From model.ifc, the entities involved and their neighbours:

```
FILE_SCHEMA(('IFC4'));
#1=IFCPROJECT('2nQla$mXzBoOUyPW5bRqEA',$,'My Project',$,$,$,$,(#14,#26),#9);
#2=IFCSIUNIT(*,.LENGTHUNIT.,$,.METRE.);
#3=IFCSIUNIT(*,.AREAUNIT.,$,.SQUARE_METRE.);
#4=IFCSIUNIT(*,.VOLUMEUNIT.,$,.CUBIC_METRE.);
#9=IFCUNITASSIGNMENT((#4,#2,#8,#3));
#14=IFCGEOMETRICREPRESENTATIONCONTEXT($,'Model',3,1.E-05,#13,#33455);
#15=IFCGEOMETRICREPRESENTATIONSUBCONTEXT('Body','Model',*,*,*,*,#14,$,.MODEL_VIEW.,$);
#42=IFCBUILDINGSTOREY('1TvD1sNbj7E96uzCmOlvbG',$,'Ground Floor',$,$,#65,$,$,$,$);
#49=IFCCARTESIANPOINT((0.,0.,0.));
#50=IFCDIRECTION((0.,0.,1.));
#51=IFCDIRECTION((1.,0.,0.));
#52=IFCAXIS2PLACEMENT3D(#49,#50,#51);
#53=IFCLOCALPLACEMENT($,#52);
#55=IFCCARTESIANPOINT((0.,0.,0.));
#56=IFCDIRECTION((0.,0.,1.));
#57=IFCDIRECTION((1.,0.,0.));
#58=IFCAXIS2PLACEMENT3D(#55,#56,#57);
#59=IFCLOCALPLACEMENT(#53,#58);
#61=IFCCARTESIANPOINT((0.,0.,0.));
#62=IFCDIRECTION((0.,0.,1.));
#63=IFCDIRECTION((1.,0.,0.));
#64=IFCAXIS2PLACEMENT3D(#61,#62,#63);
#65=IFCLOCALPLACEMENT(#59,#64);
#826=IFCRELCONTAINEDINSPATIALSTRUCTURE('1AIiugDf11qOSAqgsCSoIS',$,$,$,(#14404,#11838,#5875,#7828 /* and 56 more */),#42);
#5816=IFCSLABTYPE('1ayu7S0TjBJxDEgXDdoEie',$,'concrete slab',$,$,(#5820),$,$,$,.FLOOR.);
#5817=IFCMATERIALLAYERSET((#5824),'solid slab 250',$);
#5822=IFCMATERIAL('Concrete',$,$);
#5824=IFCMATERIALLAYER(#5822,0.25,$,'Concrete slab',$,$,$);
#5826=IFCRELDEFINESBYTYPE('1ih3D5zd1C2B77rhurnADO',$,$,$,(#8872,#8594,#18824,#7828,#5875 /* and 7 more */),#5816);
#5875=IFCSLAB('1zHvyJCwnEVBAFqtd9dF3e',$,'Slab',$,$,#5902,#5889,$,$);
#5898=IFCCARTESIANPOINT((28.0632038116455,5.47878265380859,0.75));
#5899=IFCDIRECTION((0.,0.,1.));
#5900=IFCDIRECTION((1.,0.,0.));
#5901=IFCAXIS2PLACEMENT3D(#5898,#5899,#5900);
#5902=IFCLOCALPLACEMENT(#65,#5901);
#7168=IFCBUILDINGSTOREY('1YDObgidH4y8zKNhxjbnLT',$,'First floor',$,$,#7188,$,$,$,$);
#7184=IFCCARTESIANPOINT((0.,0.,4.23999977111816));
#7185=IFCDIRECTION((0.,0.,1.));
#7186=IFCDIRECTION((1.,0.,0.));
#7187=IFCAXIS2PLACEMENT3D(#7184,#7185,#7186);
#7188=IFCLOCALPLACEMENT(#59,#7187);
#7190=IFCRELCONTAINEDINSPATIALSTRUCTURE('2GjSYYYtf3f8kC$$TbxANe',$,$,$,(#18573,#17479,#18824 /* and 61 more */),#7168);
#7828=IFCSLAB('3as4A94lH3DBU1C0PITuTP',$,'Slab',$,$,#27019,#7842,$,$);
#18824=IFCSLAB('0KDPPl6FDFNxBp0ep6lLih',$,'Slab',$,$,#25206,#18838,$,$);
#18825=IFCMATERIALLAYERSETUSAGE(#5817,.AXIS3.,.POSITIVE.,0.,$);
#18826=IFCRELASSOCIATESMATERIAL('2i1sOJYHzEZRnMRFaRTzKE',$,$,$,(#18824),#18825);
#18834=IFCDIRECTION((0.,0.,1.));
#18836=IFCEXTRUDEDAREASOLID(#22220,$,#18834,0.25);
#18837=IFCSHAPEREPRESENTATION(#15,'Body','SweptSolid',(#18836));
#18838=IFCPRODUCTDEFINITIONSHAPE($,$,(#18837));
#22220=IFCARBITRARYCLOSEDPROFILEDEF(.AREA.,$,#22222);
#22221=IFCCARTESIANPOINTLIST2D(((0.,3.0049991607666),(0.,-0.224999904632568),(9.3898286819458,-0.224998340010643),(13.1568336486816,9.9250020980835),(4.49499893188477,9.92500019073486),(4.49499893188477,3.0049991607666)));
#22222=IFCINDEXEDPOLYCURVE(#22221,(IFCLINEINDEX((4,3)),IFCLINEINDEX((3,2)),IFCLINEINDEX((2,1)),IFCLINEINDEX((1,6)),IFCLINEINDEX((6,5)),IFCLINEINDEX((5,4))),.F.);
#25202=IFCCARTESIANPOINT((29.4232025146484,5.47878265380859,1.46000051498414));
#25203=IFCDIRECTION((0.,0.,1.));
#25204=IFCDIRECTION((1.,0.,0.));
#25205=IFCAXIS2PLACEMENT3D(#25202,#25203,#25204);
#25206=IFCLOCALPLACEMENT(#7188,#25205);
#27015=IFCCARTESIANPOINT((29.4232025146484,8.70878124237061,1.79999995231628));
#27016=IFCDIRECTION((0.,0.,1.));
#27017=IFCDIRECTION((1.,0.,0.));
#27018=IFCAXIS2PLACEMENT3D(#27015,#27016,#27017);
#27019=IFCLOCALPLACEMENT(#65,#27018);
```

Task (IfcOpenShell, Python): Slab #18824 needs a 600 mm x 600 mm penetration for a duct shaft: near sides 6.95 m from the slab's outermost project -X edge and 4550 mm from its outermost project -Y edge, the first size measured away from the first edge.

```python
import numpy as np
import ifcopenshell
import ifcopenshell.api.feature
import ifcopenshell.api.geometry
import ifcopenshell.api.root
import ifcopenshell.geom
import ifcopenshell.util.placement
import ifcopenshell.util.representation
import ifcopenshell.util.shape
import ifcopenshell.util.unit

model = ifcopenshell.open("model.ifc")
unit_scale = ifcopenshell.util.unit.calculate_unit_scale(model)
settings = ifcopenshell.geom.settings()


def volume(element):
    """Net volume in cubic metres, openings subtracted."""
    shape = ifcopenshell.geom.create_shape(settings, element)
    return ifcopenshell.util.shape.get_volume(shape.geometry)


slab = model.by_guid("0KDPPl6FDFNxBp0ep6lLih")
before = volume(slab)

# Extent in the slab's own axes, in metres. The edges named are its -X and -Y sides.
slab_shape = ifcopenshell.geom.create_shape(settings, slab)
vertices = ifcopenshell.util.shape.get_vertices(slab_shape.geometry)
x_min, y_min, bottom = vertices.min(axis=0)
top = vertices[:, 2].max()

opening = ifcopenshell.api.root.create_entity(model, ifc_class="IfcOpeningElement", name="Duct shaft opening", predefined_type="OPENING")
context = ifcopenshell.util.representation.get_context(model, "Model", "Body", "MODEL_VIEW")
width, depth = 0.6, 0.6
outline = [(0.0, 0.0), (width, 0.0), (width, depth), (0.0, depth), (0.0, 0.0)]
# Overshoot both faces by 50 mm so the cut is clean.
shape = ifcopenshell.api.geometry.add_slab_representation(
    model, context=context, depth=top - bottom + 0.1, polyline=outline
)
ifcopenshell.api.geometry.assign_representation(model, product=opening, representation=shape)

matrix = ifcopenshell.util.placement.get_local_placement(slab.ObjectPlacement)
matrix[:, 3] = matrix @ np.append(np.array([x_min + 6.95, y_min + 4.55, bottom - 0.05]) / unit_scale, 1.0)
ifcopenshell.api.geometry.edit_object_placement(model, product=opening, matrix=matrix, is_si=False)
ifcopenshell.api.feature.add_feature(model, feature=opening, element=slab)

after = volume(slab)

print(f"slab volume {before:.3f} -> {after:.3f} m3")

model.write("model_updated.ifc")
```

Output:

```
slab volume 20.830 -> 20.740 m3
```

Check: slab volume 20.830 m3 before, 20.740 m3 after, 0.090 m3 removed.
